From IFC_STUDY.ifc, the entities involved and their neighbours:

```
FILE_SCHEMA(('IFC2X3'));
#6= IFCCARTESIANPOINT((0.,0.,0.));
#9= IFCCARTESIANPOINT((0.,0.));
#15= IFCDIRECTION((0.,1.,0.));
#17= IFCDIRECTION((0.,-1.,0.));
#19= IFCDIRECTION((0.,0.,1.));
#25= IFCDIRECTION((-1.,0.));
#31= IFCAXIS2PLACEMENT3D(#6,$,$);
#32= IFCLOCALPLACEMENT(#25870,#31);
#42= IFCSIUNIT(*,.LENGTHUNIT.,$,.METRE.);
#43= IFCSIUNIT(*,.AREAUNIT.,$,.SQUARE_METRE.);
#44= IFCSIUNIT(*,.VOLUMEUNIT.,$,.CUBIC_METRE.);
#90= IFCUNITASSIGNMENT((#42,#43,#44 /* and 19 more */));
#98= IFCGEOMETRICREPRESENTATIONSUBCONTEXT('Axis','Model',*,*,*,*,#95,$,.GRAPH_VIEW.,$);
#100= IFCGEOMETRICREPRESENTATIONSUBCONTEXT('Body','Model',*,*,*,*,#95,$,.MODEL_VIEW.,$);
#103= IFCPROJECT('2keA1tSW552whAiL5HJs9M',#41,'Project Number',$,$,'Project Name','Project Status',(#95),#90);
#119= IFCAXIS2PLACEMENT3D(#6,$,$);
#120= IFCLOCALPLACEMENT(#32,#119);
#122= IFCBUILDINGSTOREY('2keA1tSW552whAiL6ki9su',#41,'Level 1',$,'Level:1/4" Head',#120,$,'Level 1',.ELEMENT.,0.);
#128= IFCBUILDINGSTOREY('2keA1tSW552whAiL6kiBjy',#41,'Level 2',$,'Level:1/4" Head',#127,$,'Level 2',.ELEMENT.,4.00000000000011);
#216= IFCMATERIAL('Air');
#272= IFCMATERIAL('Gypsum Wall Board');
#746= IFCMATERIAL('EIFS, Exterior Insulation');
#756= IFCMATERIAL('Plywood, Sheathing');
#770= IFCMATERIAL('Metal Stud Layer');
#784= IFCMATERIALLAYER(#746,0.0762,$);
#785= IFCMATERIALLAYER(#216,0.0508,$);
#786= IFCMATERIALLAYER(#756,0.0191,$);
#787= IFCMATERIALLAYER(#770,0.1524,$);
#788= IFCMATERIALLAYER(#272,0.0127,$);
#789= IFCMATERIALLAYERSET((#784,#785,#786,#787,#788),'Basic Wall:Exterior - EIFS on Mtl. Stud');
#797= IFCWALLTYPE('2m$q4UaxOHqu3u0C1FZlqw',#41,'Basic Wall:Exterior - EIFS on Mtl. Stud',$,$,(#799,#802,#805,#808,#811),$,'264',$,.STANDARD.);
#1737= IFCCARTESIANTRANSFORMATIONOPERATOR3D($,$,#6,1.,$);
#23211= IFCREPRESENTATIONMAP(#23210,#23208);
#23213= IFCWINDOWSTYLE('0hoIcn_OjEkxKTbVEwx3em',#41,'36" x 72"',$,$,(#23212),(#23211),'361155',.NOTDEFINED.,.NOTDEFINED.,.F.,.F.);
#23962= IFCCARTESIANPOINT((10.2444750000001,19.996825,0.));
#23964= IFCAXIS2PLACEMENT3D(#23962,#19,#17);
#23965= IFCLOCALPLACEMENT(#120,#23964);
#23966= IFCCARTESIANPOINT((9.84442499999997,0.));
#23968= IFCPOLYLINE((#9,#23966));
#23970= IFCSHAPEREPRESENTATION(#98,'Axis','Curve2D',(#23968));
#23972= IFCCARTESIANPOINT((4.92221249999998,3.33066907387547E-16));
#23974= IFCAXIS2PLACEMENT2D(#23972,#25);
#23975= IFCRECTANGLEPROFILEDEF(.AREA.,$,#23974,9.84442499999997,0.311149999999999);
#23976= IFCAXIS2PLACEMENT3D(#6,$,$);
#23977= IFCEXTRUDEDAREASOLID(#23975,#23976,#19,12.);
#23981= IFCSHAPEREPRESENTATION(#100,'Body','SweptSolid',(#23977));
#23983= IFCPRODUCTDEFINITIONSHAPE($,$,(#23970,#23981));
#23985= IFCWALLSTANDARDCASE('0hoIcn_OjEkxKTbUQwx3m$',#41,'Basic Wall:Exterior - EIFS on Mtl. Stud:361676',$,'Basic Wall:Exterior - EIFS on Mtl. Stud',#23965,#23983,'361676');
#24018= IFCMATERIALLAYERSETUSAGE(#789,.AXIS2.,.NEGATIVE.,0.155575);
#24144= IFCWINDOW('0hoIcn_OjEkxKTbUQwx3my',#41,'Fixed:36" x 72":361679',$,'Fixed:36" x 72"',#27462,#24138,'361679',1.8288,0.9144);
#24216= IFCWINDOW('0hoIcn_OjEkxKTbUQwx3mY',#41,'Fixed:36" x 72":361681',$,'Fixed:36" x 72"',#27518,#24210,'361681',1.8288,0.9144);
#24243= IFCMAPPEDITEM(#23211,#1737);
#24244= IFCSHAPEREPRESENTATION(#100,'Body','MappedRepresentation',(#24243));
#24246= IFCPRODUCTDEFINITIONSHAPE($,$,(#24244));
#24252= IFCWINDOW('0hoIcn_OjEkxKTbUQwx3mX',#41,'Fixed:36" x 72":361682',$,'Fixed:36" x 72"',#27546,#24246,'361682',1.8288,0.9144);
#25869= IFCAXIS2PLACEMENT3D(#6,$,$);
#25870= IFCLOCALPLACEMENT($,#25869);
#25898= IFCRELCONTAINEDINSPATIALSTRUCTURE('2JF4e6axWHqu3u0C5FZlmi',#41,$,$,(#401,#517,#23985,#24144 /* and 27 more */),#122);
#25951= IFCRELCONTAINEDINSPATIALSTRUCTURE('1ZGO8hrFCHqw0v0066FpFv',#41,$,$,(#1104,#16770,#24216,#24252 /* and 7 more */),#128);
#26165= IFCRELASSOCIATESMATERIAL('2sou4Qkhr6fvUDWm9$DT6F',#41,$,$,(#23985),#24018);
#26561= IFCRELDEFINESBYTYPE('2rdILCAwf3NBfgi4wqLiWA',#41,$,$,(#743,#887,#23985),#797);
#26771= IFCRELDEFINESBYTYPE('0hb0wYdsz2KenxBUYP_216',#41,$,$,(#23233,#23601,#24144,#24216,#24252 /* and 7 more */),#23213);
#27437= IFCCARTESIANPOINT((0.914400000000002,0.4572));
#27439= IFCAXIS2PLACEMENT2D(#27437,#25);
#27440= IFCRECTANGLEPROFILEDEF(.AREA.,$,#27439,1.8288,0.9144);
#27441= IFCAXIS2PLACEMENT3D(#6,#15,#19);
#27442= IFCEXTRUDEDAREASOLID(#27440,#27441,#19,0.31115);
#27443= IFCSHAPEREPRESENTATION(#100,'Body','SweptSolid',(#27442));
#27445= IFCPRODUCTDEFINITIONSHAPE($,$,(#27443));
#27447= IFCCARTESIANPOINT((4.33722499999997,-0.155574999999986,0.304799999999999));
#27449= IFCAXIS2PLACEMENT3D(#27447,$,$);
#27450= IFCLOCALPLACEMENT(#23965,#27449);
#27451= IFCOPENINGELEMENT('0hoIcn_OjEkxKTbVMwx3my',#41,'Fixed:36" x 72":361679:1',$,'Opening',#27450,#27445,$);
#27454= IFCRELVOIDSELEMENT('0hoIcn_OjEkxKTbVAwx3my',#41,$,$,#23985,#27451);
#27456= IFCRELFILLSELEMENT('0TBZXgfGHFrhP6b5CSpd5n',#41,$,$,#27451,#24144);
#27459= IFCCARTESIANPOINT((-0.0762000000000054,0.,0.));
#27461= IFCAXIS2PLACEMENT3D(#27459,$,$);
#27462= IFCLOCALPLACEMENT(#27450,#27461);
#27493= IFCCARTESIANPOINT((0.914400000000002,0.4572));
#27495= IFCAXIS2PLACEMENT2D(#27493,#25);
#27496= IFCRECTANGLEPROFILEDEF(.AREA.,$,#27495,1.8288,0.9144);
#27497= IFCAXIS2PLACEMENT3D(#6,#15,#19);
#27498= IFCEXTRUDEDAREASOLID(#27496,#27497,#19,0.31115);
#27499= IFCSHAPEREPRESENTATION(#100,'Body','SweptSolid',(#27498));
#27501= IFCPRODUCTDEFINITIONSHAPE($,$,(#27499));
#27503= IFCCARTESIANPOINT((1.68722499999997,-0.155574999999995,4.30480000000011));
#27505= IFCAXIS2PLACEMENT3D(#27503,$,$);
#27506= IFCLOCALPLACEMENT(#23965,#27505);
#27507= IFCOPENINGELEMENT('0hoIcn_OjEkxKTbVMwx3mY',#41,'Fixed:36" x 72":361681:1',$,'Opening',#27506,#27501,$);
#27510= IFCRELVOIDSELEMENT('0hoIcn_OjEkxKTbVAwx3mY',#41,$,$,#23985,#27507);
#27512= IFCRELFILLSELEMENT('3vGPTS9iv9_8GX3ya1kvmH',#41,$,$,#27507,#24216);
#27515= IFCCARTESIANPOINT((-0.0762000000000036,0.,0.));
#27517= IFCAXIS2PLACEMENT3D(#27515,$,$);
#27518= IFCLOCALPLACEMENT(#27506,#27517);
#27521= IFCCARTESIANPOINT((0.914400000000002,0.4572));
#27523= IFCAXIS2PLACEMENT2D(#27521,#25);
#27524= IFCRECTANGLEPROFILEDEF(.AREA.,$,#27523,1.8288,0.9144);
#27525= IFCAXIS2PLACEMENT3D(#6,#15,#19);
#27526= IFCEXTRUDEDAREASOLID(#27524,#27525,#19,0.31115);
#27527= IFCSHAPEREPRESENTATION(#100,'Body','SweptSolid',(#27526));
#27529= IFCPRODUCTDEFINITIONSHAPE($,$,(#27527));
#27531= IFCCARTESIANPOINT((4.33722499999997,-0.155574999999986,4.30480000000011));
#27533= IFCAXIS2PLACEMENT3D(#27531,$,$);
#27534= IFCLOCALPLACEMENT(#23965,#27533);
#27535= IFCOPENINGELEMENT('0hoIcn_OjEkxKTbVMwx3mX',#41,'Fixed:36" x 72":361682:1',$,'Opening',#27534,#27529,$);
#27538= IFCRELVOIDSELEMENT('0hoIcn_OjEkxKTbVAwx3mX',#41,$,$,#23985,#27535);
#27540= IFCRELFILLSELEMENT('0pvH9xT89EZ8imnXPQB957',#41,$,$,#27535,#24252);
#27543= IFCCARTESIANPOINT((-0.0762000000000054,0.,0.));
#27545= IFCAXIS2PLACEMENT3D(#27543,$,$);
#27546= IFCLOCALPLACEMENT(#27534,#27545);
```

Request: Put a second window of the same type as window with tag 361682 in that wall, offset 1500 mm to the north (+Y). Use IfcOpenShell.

```python
import ifcopenshell
import ifcopenshell.api.feature
import ifcopenshell.api.geometry
import ifcopenshell.api.root
import ifcopenshell.geom
import ifcopenshell.util.element
import ifcopenshell.util.placement
import ifcopenshell.util.shape

model = ifcopenshell.open("IFC_STUDY.ifc")
settings = ifcopenshell.geom.settings()


def volume(element):
    """Net volume in cubic metres, openings subtracted."""
    shape = ifcopenshell.geom.create_shape(settings, element)
    return ifcopenshell.util.shape.get_volume(shape.geometry)


def reuse_history(source, copy):
    """copy_class also copies each property set's owner history, people and application; keep the originals."""
    for rel in copy.IsDefinedBy:
        if rel.is_a("IfcRelDefinesByProperties") and (history := rel.RelatingPropertyDefinition.OwnerHistory):
            rel.RelatingPropertyDefinition.OwnerHistory = source.OwnerHistory
            ifcopenshell.util.element.remove_deep2(model, history)


window = model.by_guid("0hoIcn_OjEkxKTbUQwx3mX")
opening = window.FillsVoids[0].RelatingOpeningElement
wall = opening.VoidsElements[0].RelatingBuildingElement
before = volume(wall)
shift = ifcopenshell.util.placement.get_local_placement(wall.ObjectPlacement)[:3, 0] * -1.5

# copy_class copies the void relationship, type, container and properties, but no geometry.
new_opening = ifcopenshell.api.root.copy_class(model, product=opening)
new_opening.Representation = ifcopenshell.util.element.copy_deep(
    model, opening.Representation, exclude=["IfcGeometricRepresentationContext", "IfcRepresentationMap"]
)
new_opening.Name = 'Fixed:36" x 72"'
new_window = ifcopenshell.api.root.copy_class(model, product=window)
new_window.Representation = ifcopenshell.util.element.copy_deep(
    model, window.Representation, exclude=["IfcGeometricRepresentationContext", "IfcRepresentationMap"]
)
new_window.Name = 'Fixed:36" x 72"'
new_window.Tag = None
reuse_history(window, new_window)
fills = ifcopenshell.api.feature.add_filling(model, opening=new_opening, element=new_window)
fills.OwnerHistory = new_window.OwnerHistory  # required in IFC2X3

for old, new in ((opening, new_opening), (window, new_window)):
    matrix = ifcopenshell.util.placement.get_local_placement(old.ObjectPlacement)
    matrix[:3, 3] += shift
    ifcopenshell.api.geometry.edit_object_placement(model, product=new, matrix=matrix, is_si=False)

after = volume(wall)

print(f"wall volume {before:.3f} -> {after:.3f} m3")

model.write("IFC_STUDY_v2.ifc")
```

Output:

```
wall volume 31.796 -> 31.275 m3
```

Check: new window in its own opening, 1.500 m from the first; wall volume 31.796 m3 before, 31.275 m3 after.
